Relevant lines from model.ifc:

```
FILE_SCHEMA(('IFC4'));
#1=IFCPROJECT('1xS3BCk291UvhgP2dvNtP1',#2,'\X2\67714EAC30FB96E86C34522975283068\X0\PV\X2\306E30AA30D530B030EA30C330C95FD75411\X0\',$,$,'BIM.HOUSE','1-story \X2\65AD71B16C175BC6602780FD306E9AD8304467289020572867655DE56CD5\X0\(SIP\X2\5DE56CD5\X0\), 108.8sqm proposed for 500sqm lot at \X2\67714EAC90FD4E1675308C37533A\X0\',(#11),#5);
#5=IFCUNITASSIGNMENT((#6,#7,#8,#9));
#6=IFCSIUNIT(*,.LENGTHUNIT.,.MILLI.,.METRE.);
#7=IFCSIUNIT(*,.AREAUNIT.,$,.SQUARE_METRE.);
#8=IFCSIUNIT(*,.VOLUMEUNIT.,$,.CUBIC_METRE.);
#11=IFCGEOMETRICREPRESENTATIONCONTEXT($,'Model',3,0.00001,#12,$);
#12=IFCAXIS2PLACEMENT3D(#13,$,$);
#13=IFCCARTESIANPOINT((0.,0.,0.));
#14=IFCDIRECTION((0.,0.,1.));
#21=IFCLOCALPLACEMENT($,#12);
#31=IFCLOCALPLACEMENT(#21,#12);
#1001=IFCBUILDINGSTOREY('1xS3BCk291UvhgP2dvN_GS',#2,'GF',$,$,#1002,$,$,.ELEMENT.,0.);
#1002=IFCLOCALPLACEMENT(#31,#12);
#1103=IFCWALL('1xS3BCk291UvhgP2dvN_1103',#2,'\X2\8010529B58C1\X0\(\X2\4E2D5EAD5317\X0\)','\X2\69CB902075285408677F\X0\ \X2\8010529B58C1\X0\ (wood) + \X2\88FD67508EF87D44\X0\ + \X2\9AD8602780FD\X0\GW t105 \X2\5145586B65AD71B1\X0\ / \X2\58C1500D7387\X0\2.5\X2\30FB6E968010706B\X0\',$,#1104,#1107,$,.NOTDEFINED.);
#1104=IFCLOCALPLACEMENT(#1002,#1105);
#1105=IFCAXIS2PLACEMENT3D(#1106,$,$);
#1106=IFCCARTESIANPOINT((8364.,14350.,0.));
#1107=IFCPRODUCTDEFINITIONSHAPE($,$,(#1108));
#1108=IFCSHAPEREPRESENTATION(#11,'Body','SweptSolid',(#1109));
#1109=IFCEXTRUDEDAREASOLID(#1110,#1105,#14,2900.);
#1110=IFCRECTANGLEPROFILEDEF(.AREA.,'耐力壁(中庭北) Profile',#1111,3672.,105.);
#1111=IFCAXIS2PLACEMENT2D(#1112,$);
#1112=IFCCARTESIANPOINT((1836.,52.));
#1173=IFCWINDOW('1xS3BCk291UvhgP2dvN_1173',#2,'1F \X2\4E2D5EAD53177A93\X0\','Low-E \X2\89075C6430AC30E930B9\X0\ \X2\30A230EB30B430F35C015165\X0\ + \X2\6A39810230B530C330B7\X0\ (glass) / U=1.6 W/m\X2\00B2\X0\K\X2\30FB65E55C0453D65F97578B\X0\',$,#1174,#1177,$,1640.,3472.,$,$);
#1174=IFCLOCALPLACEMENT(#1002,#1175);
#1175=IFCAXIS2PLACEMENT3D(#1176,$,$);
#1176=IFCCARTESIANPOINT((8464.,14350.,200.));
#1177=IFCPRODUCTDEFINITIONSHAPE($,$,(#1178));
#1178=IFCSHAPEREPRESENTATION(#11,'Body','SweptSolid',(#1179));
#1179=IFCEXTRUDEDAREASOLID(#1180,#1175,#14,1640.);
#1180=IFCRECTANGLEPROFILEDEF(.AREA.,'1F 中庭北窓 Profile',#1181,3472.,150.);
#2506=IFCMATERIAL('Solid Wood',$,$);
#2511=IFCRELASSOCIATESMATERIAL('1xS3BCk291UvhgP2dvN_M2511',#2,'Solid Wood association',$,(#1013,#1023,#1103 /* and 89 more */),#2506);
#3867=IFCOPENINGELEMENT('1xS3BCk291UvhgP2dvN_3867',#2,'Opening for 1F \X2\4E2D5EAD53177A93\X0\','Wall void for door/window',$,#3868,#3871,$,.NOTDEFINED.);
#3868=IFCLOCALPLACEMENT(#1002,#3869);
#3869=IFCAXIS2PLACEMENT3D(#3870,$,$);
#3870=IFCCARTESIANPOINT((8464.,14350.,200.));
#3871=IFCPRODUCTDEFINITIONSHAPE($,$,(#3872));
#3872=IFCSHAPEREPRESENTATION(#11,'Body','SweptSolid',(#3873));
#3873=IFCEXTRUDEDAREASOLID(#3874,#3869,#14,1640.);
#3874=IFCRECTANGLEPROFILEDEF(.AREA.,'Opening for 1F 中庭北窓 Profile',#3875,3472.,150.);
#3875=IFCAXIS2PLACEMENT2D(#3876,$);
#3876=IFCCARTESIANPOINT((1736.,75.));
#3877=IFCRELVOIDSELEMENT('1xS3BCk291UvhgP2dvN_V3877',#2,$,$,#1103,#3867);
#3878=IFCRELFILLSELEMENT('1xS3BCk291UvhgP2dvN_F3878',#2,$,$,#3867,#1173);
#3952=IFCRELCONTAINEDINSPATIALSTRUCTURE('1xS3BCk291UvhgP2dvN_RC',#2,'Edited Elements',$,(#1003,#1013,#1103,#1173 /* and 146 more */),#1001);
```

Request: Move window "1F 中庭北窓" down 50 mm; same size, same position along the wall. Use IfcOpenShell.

```python
import numpy as np
import ifcopenshell
import ifcopenshell.api.geometry
import ifcopenshell.util.placement
import ifcopenshell.util.unit

model = ifcopenshell.open("model.ifc")
unit_scale = ifcopenshell.util.unit.calculate_unit_scale(model)

window = model.by_guid("1xS3BCk291UvhgP2dvN_1173")
opening = window.FillsVoids[0].RelatingOpeningElement
dz = -0.05 / unit_scale

shift = np.array([0.0, 0.0, dz])
# The window is not placed relative to its opening, so move both.
for product in (opening, window):
    matrix = ifcopenshell.util.placement.get_local_placement(product.ObjectPlacement)
    matrix[:3, 3] += shift
    ifcopenshell.api.geometry.edit_object_placement(model, product=product, matrix=matrix, is_si=False)

print(f"moved by {dz * unit_scale:+.3f} m")

model.write("model_updated.ifc")
```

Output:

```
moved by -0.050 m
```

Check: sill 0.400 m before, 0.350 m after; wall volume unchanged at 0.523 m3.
